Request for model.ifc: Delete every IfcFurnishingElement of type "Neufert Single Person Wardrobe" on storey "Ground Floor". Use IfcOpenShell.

First a look at what the model holds.

```python
import ifcopenshell
import ifcopenshell.util.element

model = ifcopenshell.open("model.ifc")
print(model.schema)
storey = next(s for s in model.by_type("IfcBuildingStorey") if s.Name == "Ground Floor")
furniture = [e for e in ifcopenshell.util.element.get_decomposition(storey) if e.is_a("IfcFurnishingElement")]
seen = {}
for e in furniture:
    element_type = ifcopenshell.util.element.get_type(e)
    name = element_type.Name if element_type not in (None, e) else None
    seen[name] = seen.get(name, 0) + 1
for name, count in sorted(seen.items(), key=str):
    print(count, "x", name)
```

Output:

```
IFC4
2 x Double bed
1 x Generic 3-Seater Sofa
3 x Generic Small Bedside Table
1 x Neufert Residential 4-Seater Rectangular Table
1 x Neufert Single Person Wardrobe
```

```python
import ifcopenshell
import ifcopenshell.api.root
import ifcopenshell.util.element

model = ifcopenshell.open("model.ifc")

storey = next(s for s in model.by_type("IfcBuildingStorey") if s.Name == "Ground Floor")
furniture = [e for e in ifcopenshell.util.element.get_decomposition(storey) if e.is_a("IfcFurnishingElement")]
targets = [e for e in furniture if (t := ifcopenshell.util.element.get_type(e)) not in (None, e) and t.Name == "Neufert Single Person Wardrobe"]

for e in targets:
    ifcopenshell.api.root.remove_product(model, product=e)
print(len(targets), "removed")

model.write("model_v2.ifc")
```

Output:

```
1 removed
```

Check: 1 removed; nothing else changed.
